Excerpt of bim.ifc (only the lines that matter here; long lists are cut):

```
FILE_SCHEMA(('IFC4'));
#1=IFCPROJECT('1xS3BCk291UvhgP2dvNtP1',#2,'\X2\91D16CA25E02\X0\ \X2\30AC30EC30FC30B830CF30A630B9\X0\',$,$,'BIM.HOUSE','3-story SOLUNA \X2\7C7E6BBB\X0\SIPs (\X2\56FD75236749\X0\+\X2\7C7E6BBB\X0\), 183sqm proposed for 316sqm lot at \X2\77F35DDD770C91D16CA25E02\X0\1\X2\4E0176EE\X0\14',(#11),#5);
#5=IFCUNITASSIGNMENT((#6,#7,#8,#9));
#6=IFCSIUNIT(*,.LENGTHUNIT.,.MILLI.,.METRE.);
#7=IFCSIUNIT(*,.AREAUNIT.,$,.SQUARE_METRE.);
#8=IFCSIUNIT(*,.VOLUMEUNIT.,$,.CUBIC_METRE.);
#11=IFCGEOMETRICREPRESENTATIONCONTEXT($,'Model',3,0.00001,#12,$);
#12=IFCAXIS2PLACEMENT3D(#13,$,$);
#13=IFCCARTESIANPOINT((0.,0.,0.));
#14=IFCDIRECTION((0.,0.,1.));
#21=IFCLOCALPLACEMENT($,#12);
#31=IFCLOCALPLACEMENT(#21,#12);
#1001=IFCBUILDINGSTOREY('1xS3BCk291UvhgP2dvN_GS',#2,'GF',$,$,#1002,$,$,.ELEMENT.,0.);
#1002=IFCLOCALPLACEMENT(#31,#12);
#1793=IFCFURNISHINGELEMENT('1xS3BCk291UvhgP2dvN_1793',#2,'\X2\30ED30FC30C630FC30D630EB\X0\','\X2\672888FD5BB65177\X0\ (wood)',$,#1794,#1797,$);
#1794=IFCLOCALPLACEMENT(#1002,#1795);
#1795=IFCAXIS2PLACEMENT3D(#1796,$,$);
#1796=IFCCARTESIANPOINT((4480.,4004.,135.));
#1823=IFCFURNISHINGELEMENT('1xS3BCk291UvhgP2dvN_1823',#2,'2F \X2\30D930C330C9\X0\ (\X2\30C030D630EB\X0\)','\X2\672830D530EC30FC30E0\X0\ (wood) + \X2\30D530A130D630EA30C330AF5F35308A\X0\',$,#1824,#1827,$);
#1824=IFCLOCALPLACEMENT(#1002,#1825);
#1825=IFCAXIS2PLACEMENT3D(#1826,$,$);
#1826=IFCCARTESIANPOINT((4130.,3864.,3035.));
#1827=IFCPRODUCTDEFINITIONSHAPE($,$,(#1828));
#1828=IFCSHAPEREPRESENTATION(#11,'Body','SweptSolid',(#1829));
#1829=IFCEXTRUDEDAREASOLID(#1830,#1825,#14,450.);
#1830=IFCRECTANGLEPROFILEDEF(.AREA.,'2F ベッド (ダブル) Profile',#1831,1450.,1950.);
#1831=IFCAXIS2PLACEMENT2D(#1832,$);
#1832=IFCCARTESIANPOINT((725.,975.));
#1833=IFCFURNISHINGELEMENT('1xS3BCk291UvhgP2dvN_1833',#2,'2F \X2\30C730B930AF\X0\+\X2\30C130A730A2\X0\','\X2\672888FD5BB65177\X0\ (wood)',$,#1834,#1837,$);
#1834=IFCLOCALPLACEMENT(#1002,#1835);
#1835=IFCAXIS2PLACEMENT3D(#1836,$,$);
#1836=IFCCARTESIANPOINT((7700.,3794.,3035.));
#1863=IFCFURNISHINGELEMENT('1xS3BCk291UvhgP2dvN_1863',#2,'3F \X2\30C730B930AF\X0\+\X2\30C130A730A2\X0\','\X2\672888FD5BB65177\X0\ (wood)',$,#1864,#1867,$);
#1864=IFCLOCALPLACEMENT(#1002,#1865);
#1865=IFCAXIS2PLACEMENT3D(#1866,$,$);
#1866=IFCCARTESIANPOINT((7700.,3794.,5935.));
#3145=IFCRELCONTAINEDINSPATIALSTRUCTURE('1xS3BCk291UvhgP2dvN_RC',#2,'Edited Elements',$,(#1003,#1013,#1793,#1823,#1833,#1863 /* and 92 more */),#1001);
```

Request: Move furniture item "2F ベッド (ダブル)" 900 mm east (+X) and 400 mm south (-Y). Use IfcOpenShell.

```python
import ifcopenshell
import ifcopenshell.api.geometry
import ifcopenshell.util.placement
import ifcopenshell.util.unit

model = ifcopenshell.open("bim.ifc")
unit_scale = ifcopenshell.util.unit.calculate_unit_scale(model)

item = model.by_guid("1xS3BCk291UvhgP2dvN_1823")
matrix = ifcopenshell.util.placement.get_local_placement(item.ObjectPlacement)
matrix[0, 3] += 0.9 / unit_scale
matrix[1, 3] -= 0.4 / unit_scale
ifcopenshell.api.geometry.edit_object_placement(model, product=item, matrix=matrix, is_si=False)

print(ifcopenshell.util.placement.get_local_placement(item.ObjectPlacement).round(3) + 0.0)

model.write("bim-out.ifc")
```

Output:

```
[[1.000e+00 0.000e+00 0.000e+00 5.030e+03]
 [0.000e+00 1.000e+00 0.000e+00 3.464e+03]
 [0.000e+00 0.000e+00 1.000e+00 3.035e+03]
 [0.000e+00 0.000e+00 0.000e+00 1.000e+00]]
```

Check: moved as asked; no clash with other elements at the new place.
